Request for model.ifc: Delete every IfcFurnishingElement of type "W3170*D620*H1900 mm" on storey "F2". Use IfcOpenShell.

First a look at what the model holds.

```python
import ifcopenshell
import ifcopenshell.util.element

model = ifcopenshell.open("model.ifc")
print(model.schema)
storey = next(s for s in model.by_type("IfcBuildingStorey") if s.Name == "F2")
furniture = [e for e in ifcopenshell.util.element.get_decomposition(storey) if e.is_a("IfcFurnishingElement")]
seen = {}
for e in furniture:
    element_type = ifcopenshell.util.element.get_type(e)
    name = element_type.Name if element_type not in (None, e) else None
    seen[name] = seen.get(name, 0) + 1
for name, count in sorted(seen.items(), key=str):
    print(count, "x", name)
```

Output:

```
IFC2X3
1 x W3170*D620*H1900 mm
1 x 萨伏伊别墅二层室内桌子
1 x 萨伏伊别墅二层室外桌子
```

```python
import ifcopenshell
import ifcopenshell.api.root
import ifcopenshell.util.element

model = ifcopenshell.open("model.ifc")

storey = next(s for s in model.by_type("IfcBuildingStorey") if s.Name == "F2")
furniture = [e for e in ifcopenshell.util.element.get_decomposition(storey) if e.is_a("IfcFurnishingElement")]
targets = [e for e in furniture if (t := ifcopenshell.util.element.get_type(e)) not in (None, e) and t.Name == "W3170*D620*H1900 mm"]

for e in targets:
    ifcopenshell.api.root.remove_product(model, product=e)
print(len(targets), "removed")

model.write("model_updated.ifc")
```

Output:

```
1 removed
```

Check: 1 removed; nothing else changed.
